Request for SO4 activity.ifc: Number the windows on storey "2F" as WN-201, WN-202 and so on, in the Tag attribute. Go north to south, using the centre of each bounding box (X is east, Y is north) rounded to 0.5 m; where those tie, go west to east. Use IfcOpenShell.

First a look at what the model holds.

```python
import ifcopenshell
import ifcopenshell.util.element
import ifcopenshell.util.placement

model = ifcopenshell.open("SO4 activity.ifc")
print(model.schema)
storey = next(s for s in model.by_type("IfcBuildingStorey") if s.Name == "2F")
windows = [e for e in ifcopenshell.util.element.get_decomposition(storey) if e.is_a("IfcWindow")]
for e in sorted(windows, key=lambda e: e.id()):
    origin = ifcopenshell.util.placement.get_local_placement(e.ObjectPlacement)[:3, 3]
    print(e.id(), e.Tag, e.Name, origin.round(2) + 0.0, sep=" | ")
```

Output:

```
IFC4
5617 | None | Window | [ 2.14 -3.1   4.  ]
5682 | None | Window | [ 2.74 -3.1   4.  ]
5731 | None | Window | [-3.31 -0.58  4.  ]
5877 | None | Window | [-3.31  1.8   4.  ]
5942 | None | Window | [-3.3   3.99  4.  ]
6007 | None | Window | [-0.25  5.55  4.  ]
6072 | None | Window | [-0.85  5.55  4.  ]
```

```python
import ifcopenshell
import ifcopenshell.geom
import ifcopenshell.util.element
import ifcopenshell.util.shape

model = ifcopenshell.open("SO4 activity.ifc")
settings = ifcopenshell.geom.settings()
settings.set("use-world-coords", True)


def centre(element):
    shape = ifcopenshell.geom.create_shape(settings, element)
    return ifcopenshell.util.shape.get_bbox_centroid(shape.geometry)


storey = next(s for s in model.by_type("IfcBuildingStorey") if s.Name == "2F")
windows = [e for e in ifcopenshell.util.element.get_decomposition(storey) if e.is_a("IfcWindow")]

# Insertion points can sit at a corner or the storey origin, so sort by the geometry (in metres).
centres = {e: centre(e) for e in windows}
windows.sort(key=lambda e: (-round(centres[e][1] / 0.5), centres[e][0]))

for i, e in enumerate(windows, start=1):
    number = f"WN-2{i:02d}"
    e.Tag = number
    print(e.id(), number)

model.write("SO4 activity_v2.ifc")
```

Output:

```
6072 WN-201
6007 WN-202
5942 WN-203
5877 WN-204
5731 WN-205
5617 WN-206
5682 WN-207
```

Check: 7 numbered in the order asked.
